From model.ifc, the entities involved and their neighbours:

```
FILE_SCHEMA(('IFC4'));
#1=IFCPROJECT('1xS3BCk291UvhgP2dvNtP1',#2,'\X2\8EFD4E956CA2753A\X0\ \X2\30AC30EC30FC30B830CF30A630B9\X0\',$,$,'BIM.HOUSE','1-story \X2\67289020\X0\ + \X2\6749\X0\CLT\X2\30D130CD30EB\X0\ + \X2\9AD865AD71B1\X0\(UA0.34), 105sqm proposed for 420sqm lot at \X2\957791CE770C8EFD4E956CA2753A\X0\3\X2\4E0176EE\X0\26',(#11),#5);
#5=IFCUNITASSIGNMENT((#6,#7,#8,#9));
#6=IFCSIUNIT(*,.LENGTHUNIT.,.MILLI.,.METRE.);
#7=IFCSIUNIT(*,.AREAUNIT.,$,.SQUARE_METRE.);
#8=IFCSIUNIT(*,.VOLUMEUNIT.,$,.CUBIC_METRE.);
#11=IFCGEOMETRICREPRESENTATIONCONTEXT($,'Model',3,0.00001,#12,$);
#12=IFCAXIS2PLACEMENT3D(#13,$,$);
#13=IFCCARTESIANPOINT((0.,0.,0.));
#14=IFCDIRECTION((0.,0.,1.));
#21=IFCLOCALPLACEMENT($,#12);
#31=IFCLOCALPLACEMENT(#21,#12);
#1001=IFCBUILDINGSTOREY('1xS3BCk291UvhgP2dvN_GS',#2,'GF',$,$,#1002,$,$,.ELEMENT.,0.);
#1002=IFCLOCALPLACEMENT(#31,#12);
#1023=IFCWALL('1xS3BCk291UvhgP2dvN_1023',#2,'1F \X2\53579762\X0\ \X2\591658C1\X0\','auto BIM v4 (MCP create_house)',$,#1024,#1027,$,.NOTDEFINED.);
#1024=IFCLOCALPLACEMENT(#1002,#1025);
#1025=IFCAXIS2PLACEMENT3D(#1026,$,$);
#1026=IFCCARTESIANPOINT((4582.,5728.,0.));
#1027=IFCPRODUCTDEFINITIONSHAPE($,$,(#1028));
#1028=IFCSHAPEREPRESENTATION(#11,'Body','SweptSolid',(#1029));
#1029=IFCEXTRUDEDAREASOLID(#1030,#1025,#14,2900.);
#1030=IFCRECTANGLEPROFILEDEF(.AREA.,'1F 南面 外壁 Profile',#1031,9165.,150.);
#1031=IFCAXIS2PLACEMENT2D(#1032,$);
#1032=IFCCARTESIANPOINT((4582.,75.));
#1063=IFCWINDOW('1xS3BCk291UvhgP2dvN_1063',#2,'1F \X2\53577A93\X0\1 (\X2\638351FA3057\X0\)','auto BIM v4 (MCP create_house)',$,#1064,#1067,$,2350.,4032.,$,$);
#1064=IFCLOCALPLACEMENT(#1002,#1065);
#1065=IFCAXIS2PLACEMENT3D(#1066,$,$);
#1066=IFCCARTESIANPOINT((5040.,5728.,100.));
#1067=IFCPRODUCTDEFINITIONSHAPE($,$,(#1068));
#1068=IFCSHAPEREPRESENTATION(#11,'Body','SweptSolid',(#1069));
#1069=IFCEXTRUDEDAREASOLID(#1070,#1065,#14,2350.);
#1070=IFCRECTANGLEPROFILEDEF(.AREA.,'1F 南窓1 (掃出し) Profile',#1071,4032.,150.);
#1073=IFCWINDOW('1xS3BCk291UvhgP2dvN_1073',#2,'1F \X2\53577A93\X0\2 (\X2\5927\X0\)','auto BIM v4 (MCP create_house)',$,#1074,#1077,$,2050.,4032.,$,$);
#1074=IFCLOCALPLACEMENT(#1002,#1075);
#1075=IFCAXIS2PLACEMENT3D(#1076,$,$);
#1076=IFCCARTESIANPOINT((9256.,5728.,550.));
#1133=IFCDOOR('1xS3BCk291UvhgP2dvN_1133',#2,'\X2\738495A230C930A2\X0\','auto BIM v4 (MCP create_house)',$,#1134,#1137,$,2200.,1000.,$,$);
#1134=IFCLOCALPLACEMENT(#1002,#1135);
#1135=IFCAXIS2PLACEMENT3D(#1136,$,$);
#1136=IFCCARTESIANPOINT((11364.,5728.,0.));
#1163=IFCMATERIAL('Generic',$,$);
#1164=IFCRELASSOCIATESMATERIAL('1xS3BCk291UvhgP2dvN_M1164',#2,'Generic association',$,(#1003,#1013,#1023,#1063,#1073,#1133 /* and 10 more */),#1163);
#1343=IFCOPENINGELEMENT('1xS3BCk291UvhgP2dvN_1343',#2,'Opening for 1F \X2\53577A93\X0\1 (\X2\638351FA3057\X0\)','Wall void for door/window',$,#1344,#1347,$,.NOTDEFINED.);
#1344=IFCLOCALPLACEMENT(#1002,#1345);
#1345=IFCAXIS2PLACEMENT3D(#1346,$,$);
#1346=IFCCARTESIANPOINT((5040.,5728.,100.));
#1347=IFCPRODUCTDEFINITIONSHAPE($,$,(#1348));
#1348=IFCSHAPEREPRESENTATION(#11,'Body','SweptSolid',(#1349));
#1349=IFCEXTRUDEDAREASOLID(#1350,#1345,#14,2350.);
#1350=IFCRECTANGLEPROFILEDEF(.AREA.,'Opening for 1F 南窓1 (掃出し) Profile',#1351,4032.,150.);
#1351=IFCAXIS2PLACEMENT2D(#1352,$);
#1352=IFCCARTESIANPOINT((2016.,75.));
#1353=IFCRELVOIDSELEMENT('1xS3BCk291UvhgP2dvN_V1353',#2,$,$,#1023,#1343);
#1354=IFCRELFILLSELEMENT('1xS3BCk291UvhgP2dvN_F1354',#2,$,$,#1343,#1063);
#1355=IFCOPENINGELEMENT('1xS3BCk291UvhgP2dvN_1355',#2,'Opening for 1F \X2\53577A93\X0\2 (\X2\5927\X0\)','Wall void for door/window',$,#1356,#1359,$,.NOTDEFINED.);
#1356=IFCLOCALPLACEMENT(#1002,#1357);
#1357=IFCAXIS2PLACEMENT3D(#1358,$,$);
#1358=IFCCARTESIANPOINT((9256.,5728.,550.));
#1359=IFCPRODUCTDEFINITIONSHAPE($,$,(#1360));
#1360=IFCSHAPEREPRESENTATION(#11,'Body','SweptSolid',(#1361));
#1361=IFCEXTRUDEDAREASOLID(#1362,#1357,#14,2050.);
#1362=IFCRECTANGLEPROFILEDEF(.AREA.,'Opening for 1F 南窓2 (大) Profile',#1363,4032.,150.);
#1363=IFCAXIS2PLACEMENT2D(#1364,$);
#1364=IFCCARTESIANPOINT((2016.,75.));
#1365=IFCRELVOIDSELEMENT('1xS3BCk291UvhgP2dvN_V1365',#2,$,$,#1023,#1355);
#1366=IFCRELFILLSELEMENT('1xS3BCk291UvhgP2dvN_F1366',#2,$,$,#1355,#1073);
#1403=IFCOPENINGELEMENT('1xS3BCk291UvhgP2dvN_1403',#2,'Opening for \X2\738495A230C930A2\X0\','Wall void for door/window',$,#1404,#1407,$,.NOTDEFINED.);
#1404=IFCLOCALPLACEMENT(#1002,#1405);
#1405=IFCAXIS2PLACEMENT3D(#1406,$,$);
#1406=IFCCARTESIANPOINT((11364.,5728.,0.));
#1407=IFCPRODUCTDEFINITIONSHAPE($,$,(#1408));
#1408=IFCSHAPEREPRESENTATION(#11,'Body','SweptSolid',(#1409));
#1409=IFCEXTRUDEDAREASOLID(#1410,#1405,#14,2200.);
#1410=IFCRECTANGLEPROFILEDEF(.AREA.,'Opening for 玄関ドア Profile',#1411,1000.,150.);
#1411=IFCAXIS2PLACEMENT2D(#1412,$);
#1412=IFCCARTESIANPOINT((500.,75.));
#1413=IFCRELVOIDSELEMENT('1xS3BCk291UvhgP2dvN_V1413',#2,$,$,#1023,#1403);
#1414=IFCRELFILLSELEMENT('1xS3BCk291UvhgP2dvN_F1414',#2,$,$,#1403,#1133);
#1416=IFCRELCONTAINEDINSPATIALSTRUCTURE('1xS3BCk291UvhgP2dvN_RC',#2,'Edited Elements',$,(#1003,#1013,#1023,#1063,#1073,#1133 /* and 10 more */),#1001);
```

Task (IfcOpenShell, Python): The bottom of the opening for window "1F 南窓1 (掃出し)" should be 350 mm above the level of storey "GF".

```python
import numpy as np
import ifcopenshell
import ifcopenshell.api.geometry
import ifcopenshell.geom
import ifcopenshell.util.element
import ifcopenshell.util.placement
import ifcopenshell.util.shape
import ifcopenshell.util.unit

model = ifcopenshell.open("model.ifc")
unit_scale = ifcopenshell.util.unit.calculate_unit_scale(model)

window = model.by_guid("1xS3BCk291UvhgP2dvN_1063")
opening = window.FillsVoids[0].RelatingOpeningElement
storey = ifcopenshell.util.element.get_container(window, ifc_class="IfcBuildingStorey")
level = ifcopenshell.util.placement.get_local_placement(storey.ObjectPlacement)[2, 3]

# The opening's origin need not be at the sill, so measure its lowest point.
shape = ifcopenshell.geom.create_shape(ifcopenshell.geom.settings(), opening)
bottom = ifcopenshell.util.shape.get_shape_bottom_elevation(shape, shape.geometry) / unit_scale
dz = level + 350.0 - bottom

shift = np.array([0.0, 0.0, dz])
# The window is not placed relative to its opening, so move both.
for product in (opening, window):
    matrix = ifcopenshell.util.placement.get_local_placement(product.ObjectPlacement)
    matrix[:3, 3] += shift
    ifcopenshell.api.geometry.edit_object_placement(model, product=product, matrix=matrix, is_si=False)

print(f"moved by {dz * unit_scale:+.3f} m")

model.write("model_rev.ifc")
```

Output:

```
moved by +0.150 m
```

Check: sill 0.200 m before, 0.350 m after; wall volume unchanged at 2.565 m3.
